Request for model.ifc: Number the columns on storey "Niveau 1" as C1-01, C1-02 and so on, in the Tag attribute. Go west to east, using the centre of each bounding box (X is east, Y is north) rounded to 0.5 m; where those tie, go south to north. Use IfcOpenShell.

First a look at what the model holds.

```python
import ifcopenshell
import ifcopenshell.util.element
import ifcopenshell.util.placement

model = ifcopenshell.open("model.ifc")
print(model.schema)
storey = next(s for s in model.by_type("IfcBuildingStorey") if s.Name == "Niveau 1")
columns = [e for e in ifcopenshell.util.element.get_decomposition(storey) if e.is_a("IfcColumn")]
for e in sorted(columns, key=lambda e: e.id()):
    origin = ifcopenshell.util.placement.get_local_placement(e.ObjectPlacement)[:3, 3]
    print(e.id(), e.Tag, e.Name, origin.round(2) + 0.0, sep=" | ")
```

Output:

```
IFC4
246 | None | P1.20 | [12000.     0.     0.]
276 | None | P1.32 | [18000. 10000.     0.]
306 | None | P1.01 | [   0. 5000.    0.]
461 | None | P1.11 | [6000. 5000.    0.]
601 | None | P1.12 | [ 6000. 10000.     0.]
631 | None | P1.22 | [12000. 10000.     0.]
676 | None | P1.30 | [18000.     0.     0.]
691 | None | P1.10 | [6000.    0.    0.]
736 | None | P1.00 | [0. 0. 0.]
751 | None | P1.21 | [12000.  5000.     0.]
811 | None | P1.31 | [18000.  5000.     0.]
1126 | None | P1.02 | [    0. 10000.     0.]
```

```python
import ifcopenshell
import ifcopenshell.geom
import ifcopenshell.util.element
import ifcopenshell.util.shape

model = ifcopenshell.open("model.ifc")
settings = ifcopenshell.geom.settings()
settings.set("use-world-coords", True)


def centre(element):
    shape = ifcopenshell.geom.create_shape(settings, element)
    return ifcopenshell.util.shape.get_bbox_centroid(shape.geometry)


storey = next(s for s in model.by_type("IfcBuildingStorey") if s.Name == "Niveau 1")
columns = [e for e in ifcopenshell.util.element.get_decomposition(storey) if e.is_a("IfcColumn")]

# Insertion points can sit at a corner or the storey origin, so sort by the geometry (in metres).
centres = {e: centre(e) for e in columns}
columns.sort(key=lambda e: (round(centres[e][0] / 0.5), centres[e][1]))

for i, e in enumerate(columns, start=1):
    number = f"C1-{i:02d}"
    e.Tag = number
    print(e.id(), number)

model.write("model_rev.ifc")
```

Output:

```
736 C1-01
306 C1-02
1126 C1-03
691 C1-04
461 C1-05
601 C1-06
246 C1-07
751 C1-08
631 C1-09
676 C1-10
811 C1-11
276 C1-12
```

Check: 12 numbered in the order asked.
